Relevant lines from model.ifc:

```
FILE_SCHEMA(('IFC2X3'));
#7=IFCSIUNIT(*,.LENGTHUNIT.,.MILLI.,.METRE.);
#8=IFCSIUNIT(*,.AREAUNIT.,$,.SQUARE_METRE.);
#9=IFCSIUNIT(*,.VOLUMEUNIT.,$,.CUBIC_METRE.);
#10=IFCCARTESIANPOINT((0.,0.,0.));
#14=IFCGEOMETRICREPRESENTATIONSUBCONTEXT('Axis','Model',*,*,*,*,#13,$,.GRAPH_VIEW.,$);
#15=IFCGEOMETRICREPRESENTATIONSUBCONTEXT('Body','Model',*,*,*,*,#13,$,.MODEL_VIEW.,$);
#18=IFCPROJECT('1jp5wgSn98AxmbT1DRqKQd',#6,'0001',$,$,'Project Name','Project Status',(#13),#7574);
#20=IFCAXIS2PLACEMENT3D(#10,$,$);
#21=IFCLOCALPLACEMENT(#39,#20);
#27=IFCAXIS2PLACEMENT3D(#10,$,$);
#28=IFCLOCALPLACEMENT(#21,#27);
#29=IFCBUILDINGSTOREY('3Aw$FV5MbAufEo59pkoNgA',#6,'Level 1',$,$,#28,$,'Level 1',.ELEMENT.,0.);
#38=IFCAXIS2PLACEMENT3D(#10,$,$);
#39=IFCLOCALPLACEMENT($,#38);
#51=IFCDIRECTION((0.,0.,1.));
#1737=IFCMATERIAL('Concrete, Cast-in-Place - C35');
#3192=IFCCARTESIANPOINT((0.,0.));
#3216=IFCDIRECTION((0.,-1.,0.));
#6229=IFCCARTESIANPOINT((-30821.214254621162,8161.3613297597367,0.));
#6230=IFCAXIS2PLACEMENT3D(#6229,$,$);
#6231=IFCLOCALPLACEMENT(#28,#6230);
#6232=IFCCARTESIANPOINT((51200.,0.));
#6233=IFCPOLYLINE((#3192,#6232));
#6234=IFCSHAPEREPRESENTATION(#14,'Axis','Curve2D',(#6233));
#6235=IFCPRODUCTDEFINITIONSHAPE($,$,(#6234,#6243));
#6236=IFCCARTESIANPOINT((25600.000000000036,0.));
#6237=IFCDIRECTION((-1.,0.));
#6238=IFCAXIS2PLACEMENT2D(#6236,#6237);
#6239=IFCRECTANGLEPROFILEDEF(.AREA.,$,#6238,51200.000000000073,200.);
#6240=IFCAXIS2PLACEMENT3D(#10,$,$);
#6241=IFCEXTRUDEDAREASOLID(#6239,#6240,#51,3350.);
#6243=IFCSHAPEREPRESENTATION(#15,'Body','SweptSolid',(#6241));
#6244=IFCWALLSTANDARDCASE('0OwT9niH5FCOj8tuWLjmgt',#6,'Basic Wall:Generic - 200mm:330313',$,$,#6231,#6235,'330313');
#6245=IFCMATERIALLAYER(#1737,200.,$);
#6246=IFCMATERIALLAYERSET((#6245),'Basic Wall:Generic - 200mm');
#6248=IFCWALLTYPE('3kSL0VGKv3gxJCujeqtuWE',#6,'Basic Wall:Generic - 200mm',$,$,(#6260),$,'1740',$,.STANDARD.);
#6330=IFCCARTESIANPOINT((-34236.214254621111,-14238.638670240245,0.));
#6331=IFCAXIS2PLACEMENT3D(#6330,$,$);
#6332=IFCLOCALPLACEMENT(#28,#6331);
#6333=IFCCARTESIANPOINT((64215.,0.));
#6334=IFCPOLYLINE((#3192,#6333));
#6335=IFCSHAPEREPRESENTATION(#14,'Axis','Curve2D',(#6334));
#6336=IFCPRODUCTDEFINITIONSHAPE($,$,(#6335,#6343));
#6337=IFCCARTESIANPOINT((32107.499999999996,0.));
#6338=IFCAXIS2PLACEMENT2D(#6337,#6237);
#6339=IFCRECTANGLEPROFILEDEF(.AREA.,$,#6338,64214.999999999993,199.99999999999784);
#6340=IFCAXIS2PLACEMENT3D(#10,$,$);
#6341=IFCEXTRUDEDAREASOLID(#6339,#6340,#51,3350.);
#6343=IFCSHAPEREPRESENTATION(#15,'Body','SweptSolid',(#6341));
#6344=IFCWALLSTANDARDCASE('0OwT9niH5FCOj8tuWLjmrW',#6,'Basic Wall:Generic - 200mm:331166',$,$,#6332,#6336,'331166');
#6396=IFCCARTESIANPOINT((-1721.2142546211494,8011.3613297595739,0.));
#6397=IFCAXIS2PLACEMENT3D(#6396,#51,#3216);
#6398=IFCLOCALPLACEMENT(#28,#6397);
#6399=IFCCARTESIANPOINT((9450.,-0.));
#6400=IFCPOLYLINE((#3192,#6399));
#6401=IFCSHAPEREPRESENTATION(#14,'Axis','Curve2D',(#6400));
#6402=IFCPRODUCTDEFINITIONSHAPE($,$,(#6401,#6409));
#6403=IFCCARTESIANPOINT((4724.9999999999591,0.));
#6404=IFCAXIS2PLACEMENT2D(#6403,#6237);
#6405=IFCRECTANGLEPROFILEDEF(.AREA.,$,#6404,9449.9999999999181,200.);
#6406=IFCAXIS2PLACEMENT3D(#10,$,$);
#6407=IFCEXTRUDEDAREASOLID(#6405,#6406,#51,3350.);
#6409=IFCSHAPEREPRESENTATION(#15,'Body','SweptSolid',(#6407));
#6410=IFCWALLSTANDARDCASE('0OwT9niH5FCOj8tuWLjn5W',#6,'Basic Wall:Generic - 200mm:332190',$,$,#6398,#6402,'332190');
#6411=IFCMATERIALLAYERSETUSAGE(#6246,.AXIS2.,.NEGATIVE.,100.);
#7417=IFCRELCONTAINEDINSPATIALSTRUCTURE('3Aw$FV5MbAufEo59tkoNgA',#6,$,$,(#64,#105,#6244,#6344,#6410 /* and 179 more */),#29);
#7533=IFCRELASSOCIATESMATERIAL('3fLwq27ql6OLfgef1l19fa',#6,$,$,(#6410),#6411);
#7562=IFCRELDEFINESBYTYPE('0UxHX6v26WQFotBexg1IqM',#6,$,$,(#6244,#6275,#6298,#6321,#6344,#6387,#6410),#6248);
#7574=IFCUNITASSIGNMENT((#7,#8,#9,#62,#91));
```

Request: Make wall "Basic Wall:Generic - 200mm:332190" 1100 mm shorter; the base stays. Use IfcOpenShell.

```python
import ifcopenshell
import ifcopenshell.geom
import ifcopenshell.util.representation
import ifcopenshell.util.shape
import ifcopenshell.util.unit

model = ifcopenshell.open("model.ifc")
unit_scale = ifcopenshell.util.unit.calculate_unit_scale(model)
settings = ifcopenshell.geom.settings()


def volume(element):
    """Net volume in cubic metres, openings subtracted."""
    shape = ifcopenshell.geom.create_shape(settings, element)
    return ifcopenshell.util.shape.get_volume(shape.geometry)


wall = model.by_guid("0OwT9niH5FCOj8tuWLjn5W")
before = volume(wall)

body = ifcopenshell.util.representation.get_representation(wall, "Model", "Body")
solid = body.Items[0]
old_height = solid.Depth
solid.Depth -= 1.1 / unit_scale
after = volume(wall)

print(f"height {old_height:g} -> {solid.Depth:g}, volume {before:.3f} -> {after:.3f} m3")

model.write("model_v2.ifc")
```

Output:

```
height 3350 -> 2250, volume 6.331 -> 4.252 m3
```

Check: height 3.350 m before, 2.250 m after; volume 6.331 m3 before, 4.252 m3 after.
